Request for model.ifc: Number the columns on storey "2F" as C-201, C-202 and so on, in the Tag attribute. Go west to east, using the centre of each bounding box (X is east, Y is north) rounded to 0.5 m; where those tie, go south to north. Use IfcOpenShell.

First a look at what the model holds.

```python
import ifcopenshell
import ifcopenshell.util.element
import ifcopenshell.util.placement

model = ifcopenshell.open("model.ifc")
print(model.schema)
storey = next(s for s in model.by_type("IfcBuildingStorey") if s.Name == "2F")
columns = [e for e in ifcopenshell.util.element.get_decomposition(storey) if e.is_a("IfcColumn")]
for e in sorted(columns, key=lambda e: e.id()):
    origin = ifcopenshell.util.placement.get_local_placement(e.ObjectPlacement)[:3, 3]
    print(e.id(), e.Tag, e.Name, origin.round(2) + 0.0, sep=" | ")
```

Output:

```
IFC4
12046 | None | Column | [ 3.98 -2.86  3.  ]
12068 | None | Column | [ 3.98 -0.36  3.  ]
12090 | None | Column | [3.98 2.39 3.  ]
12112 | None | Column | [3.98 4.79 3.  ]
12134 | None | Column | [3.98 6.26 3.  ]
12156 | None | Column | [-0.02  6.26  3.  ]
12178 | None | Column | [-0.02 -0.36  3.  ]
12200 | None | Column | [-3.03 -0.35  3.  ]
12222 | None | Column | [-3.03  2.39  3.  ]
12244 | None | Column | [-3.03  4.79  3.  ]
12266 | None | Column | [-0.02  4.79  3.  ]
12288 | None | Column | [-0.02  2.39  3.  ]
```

```python
import ifcopenshell
import ifcopenshell.geom
import ifcopenshell.util.element
import ifcopenshell.util.shape

model = ifcopenshell.open("model.ifc")
settings = ifcopenshell.geom.settings()
settings.set("use-world-coords", True)


def centre(element):
    shape = ifcopenshell.geom.create_shape(settings, element)
    return ifcopenshell.util.shape.get_bbox_centroid(shape.geometry)


storey = next(s for s in model.by_type("IfcBuildingStorey") if s.Name == "2F")
columns = [e for e in ifcopenshell.util.element.get_decomposition(storey) if e.is_a("IfcColumn")]

# Insertion points can sit at a corner or the storey origin, so sort by the geometry (in metres).
centres = {e: centre(e) for e in columns}
columns.sort(key=lambda e: (round(centres[e][0] / 0.5), centres[e][1]))

for i, e in enumerate(columns, start=1):
    number = f"C-2{i:02d}"
    e.Tag = number
    print(e.id(), number)

model.write("model-out.ifc")
```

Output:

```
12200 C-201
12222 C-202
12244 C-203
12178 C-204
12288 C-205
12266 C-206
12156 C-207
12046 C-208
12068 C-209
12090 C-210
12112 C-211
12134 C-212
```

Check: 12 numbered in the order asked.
